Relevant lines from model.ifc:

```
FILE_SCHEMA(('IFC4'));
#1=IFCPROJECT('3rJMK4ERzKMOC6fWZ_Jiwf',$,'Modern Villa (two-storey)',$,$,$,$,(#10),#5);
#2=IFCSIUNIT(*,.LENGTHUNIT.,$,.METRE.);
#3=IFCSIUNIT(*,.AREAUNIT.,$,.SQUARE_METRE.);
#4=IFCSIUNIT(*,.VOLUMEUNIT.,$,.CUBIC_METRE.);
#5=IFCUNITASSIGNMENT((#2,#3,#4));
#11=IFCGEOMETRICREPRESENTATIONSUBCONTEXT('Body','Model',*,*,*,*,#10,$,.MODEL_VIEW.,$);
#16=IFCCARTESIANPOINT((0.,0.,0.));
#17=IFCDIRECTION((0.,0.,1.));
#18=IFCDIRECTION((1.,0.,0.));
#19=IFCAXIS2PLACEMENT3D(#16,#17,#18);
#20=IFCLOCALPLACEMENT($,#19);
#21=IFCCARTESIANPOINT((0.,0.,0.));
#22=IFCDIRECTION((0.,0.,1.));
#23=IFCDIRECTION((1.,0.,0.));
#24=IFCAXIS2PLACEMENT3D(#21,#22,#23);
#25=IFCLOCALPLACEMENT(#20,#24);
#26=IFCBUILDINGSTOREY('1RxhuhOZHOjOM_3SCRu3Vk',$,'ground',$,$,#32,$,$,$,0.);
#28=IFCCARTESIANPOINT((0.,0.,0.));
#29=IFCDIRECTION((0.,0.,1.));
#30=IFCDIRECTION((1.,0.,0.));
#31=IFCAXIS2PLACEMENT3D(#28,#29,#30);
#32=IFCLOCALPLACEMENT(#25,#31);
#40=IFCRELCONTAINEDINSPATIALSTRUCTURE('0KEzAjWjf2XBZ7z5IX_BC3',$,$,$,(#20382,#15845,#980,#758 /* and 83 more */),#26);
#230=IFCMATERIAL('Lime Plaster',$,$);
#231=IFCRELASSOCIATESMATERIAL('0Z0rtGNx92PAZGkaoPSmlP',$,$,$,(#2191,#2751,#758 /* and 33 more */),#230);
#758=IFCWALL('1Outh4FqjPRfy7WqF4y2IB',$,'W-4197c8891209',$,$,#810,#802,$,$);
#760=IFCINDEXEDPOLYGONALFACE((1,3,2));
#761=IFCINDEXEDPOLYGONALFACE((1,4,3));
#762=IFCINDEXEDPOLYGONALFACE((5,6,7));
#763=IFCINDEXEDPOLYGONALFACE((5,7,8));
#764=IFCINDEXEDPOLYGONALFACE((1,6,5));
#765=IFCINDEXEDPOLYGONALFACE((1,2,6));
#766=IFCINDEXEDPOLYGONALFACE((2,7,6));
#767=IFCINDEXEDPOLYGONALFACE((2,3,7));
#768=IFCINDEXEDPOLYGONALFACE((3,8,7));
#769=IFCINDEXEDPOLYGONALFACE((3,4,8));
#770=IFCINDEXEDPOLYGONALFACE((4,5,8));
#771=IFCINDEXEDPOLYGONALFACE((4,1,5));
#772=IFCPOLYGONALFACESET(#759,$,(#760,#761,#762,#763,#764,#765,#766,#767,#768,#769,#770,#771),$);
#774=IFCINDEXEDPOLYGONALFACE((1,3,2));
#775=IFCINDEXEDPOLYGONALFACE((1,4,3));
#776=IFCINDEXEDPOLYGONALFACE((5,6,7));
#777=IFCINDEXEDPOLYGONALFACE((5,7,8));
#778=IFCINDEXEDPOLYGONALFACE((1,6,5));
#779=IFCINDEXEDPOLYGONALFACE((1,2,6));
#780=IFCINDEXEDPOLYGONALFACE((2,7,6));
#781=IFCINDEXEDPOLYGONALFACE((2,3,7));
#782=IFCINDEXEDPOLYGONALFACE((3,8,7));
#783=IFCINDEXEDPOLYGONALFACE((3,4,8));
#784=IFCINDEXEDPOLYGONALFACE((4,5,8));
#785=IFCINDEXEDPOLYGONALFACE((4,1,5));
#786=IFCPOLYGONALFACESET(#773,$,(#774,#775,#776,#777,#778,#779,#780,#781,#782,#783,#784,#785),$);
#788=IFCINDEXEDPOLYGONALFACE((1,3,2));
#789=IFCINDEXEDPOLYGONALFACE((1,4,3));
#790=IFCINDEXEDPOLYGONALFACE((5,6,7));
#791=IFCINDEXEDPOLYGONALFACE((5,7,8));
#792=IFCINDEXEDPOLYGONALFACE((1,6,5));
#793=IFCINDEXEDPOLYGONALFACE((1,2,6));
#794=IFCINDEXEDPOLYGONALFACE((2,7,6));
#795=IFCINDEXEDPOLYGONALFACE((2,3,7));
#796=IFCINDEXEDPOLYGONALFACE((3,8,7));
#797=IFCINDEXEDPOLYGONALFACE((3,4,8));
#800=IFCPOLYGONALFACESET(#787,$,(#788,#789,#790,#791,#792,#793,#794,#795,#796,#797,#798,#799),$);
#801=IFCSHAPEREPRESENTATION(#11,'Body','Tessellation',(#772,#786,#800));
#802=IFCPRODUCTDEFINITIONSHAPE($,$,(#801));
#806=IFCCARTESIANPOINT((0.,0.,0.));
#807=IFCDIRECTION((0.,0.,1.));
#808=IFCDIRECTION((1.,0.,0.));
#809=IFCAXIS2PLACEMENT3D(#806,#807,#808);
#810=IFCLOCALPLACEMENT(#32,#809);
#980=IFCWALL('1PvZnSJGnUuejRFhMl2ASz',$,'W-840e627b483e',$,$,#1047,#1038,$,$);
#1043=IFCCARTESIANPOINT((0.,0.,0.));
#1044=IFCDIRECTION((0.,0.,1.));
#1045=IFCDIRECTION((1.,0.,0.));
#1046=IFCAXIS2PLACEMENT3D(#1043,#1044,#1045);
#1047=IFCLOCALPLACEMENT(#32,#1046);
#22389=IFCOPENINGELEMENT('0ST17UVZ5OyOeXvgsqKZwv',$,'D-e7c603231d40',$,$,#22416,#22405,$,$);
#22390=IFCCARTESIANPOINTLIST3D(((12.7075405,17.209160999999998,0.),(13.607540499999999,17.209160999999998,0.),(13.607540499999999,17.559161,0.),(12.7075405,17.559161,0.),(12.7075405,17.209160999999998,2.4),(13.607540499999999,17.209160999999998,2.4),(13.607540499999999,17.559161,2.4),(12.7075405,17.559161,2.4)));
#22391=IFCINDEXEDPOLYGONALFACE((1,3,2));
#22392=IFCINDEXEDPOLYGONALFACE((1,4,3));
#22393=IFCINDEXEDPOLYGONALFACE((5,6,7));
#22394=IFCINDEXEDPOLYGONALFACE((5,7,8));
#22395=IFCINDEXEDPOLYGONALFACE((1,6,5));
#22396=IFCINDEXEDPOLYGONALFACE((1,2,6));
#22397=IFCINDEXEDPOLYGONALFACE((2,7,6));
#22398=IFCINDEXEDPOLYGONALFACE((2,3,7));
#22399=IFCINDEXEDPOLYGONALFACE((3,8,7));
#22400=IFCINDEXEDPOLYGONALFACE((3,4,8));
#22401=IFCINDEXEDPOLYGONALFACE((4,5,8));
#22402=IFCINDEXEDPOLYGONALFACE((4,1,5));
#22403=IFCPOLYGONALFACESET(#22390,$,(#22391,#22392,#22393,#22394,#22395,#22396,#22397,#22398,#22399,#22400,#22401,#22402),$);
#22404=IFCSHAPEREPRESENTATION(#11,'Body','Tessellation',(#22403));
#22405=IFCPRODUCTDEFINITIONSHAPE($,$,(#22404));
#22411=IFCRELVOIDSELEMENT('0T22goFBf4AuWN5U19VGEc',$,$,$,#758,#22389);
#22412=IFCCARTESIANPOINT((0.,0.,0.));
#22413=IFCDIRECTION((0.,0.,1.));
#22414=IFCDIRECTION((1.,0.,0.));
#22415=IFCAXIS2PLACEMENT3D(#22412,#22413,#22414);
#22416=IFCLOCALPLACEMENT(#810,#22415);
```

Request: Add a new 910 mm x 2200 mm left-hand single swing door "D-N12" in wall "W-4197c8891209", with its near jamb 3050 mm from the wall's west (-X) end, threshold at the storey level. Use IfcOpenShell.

```python
import numpy as np
import ifcopenshell
import ifcopenshell.api.feature
import ifcopenshell.api.geometry
import ifcopenshell.api.root
import ifcopenshell.api.spatial
import ifcopenshell.geom
import ifcopenshell.util.element
import ifcopenshell.util.placement
import ifcopenshell.util.representation
import ifcopenshell.util.shape
import ifcopenshell.util.unit

model = ifcopenshell.open("model.ifc")
unit_scale = ifcopenshell.util.unit.calculate_unit_scale(model)
settings = ifcopenshell.geom.settings()


def volume(element):
    """Net volume in cubic metres, openings subtracted."""
    shape = ifcopenshell.geom.create_shape(settings, element)
    return ifcopenshell.util.shape.get_volume(shape.geometry)


wall = model.by_guid("1Outh4FqjPRfy7WqF4y2IB")
storey = ifcopenshell.util.element.get_container(wall, ifc_class="IfcBuildingStorey")
context = ifcopenshell.util.representation.get_context(model, "Model", "Body", "MODEL_VIEW")
before = volume(wall)

width, height, from_end, sill = 0.91, 2.2, 3.05, 0.0  # metres

# The wall runs along its own X axis, and the end named is its -X end.
wall_shape = ifcopenshell.geom.create_shape(settings, wall)
x, y, z = ifcopenshell.util.shape.get_vertices(wall_shape.geometry).T
start = x.min() + from_end
face, thickness = float(y.min()), float(y.max() - y.min())
wall_matrix = ifcopenshell.util.placement.get_local_placement(wall.ObjectPlacement)
level = ifcopenshell.util.placement.get_local_placement(storey.ObjectPlacement)[2, 3]


def in_wall(x, y):
    """Placement at x, y metres in the wall's axes, at sill height."""
    matrix = wall_matrix.copy()
    matrix[:, 3] = wall_matrix @ np.array([x / unit_scale, y / unit_scale, 0.0, 1.0])
    matrix[2, 3] = level + sill / unit_scale
    return matrix


# Opening: a box that overshoots both wall faces by 50 mm.
opening = ifcopenshell.api.root.create_entity(model, ifc_class="IfcOpeningElement", predefined_type="OPENING")
box = ifcopenshell.api.geometry.add_wall_representation(
    model, context=context, length=width, height=height, thickness=thickness + 0.1
)
ifcopenshell.api.geometry.assign_representation(model, product=opening, representation=box)
ifcopenshell.api.geometry.edit_object_placement(model, product=opening, matrix=in_wall(start, face - 0.05), is_si=False)
ifcopenshell.api.feature.add_feature(model, feature=opening, element=wall)

door = ifcopenshell.api.root.create_entity(model, ifc_class="IfcDoor", name="D-N12", predefined_type="DOOR")
door.OverallWidth, door.OverallHeight = width / unit_scale, height / unit_scale
door.OperationType = "SINGLE_SWING_LEFT"
body = ifcopenshell.api.geometry.add_door_representation(
    model,
    context=context,
    overall_width=door.OverallWidth,
    overall_height=door.OverallHeight,
    operation_type="SINGLE_SWING_LEFT",
    lining_properties={"LiningDepth": thickness / unit_scale, "ThresholdDepth": thickness / unit_scale},
)
ifcopenshell.api.geometry.assign_representation(model, product=door, representation=body)
ifcopenshell.api.spatial.assign_container(model, products=[door], relating_structure=storey)
ifcopenshell.api.feature.add_filling(model, opening=opening, element=door)

# The lining spans the wall, so the door starts at the wall face.
ifcopenshell.api.geometry.edit_object_placement(model, product=door, matrix=in_wall(start, face), is_si=False)

after = volume(wall)

print(f"wall volume {before:.3f} -> {after:.3f} m3")

model.write("model_edited.ifc")
```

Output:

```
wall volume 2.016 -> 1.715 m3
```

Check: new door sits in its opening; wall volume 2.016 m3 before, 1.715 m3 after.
